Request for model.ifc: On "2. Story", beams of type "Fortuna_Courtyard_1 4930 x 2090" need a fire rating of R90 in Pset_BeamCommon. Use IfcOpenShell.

First a look at what the model holds.

```python
import ifcopenshell
import ifcopenshell.util.element

model = ifcopenshell.open("model.ifc")
print(model.schema)
storey = next(s for s in model.by_type("IfcBuildingStorey") if s.Name == "2. Story")
beams = [e for e in ifcopenshell.util.element.get_decomposition(storey) if e.is_a("IfcBeam")]
seen = {}
for e in beams:
    element_type = ifcopenshell.util.element.get_type(e)
    key = (element_type.Name if element_type != e and element_type else None, ifcopenshell.util.element.get_pset(e, "Pset_BeamCommon", "FireRating"))
    seen[key] = seen.get(key, 0) + 1
for (name, value), count in sorted(seen.items(), key=str):
    print(count, "x", name, "|", value)
```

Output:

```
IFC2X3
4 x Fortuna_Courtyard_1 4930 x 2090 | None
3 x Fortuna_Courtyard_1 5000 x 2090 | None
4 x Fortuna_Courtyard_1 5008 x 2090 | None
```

```python
import ifcopenshell
import ifcopenshell.api.pset
import ifcopenshell.util.element

model = ifcopenshell.open("model.ifc")

storey = next(s for s in model.by_type("IfcBuildingStorey") if s.Name == "2. Story")
beams = [e for e in ifcopenshell.util.element.get_decomposition(storey) if e.is_a("IfcBeam")]

count = 0
for e in beams:
    element_type = ifcopenshell.util.element.get_type(e)
    if element_type in (None, e) or element_type.Name != "Fortuna_Courtyard_1 4930 x 2090":
        continue
    # add_pset returns the element's existing set when there is one.
    pset = ifcopenshell.api.pset.add_pset(model, product=e, name="Pset_BeamCommon")
    ifcopenshell.api.pset.edit_pset(model, pset=pset, properties={"FireRating": "R90"})
    count += 1

print(count, "beams updated")

model.write("model_rev.ifc")
```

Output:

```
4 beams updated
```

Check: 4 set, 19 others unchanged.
